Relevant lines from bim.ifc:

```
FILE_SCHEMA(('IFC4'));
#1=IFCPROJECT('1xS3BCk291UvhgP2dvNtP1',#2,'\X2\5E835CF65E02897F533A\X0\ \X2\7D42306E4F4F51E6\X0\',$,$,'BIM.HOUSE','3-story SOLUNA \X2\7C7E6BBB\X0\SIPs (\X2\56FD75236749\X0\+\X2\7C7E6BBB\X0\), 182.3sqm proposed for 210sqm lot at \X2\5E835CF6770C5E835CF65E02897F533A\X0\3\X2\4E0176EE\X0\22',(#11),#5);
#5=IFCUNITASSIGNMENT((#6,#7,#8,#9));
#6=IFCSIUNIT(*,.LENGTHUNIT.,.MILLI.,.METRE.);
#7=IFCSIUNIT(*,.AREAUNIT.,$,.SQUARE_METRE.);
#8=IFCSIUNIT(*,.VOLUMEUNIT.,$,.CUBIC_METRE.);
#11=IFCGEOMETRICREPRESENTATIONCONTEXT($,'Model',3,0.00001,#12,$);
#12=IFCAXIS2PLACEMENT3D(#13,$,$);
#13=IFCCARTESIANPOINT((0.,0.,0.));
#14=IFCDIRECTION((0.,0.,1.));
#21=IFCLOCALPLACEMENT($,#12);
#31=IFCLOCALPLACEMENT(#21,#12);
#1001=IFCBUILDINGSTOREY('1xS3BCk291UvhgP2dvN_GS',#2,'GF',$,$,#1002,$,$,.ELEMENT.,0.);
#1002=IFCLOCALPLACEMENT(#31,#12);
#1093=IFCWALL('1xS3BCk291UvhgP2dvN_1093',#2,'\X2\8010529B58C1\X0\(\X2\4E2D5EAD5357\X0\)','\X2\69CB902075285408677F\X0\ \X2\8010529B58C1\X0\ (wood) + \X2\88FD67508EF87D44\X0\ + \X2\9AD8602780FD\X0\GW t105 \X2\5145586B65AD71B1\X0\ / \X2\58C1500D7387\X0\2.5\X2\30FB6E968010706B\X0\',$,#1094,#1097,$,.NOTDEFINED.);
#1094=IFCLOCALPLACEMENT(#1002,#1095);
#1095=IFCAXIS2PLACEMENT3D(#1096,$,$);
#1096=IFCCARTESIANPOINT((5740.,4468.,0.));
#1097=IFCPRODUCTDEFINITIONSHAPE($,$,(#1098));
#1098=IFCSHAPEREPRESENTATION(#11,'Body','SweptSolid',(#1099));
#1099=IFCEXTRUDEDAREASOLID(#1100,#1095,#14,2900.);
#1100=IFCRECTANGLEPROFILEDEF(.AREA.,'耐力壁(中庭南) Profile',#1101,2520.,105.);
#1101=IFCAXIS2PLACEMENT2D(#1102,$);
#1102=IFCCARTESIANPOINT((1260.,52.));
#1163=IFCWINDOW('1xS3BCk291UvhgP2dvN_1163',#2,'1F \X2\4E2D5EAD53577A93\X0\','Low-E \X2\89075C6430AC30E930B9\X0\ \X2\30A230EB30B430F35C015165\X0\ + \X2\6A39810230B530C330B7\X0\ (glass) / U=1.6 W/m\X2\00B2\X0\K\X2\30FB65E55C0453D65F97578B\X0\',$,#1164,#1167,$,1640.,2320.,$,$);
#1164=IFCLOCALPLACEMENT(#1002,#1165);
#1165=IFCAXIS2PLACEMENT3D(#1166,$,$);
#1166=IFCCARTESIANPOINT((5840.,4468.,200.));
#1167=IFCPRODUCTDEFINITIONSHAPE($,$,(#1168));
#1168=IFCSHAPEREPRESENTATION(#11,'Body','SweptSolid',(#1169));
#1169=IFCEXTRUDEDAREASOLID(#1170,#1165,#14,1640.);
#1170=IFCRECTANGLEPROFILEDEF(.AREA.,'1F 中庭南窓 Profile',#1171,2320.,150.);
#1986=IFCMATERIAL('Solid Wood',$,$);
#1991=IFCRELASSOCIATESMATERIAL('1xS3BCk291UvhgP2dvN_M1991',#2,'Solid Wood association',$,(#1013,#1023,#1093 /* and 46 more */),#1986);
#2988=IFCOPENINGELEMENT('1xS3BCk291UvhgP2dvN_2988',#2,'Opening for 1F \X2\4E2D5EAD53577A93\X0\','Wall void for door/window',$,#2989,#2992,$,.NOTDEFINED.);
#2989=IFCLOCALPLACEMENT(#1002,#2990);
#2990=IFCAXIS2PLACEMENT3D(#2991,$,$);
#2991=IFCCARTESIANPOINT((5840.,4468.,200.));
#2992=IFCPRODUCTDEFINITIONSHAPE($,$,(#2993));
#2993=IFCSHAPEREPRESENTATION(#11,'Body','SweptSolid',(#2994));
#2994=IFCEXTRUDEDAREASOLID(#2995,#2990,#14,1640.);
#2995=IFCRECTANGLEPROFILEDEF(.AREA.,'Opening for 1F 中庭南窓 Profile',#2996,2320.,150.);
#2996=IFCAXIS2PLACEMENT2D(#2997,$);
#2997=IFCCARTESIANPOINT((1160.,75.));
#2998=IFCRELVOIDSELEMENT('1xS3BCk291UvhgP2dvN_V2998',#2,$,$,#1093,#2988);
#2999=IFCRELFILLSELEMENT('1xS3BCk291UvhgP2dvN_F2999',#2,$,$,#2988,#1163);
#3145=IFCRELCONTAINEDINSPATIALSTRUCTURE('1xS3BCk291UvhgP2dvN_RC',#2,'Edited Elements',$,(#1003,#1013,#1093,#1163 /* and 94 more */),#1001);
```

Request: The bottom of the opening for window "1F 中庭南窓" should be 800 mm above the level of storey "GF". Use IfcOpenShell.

```python
import numpy as np
import ifcopenshell
import ifcopenshell.api.geometry
import ifcopenshell.geom
import ifcopenshell.util.element
import ifcopenshell.util.placement
import ifcopenshell.util.shape
import ifcopenshell.util.unit

model = ifcopenshell.open("bim.ifc")
unit_scale = ifcopenshell.util.unit.calculate_unit_scale(model)

window = model.by_guid("1xS3BCk291UvhgP2dvN_1163")
opening = window.FillsVoids[0].RelatingOpeningElement
storey = ifcopenshell.util.element.get_container(window, ifc_class="IfcBuildingStorey")
level = ifcopenshell.util.placement.get_local_placement(storey.ObjectPlacement)[2, 3]

# The opening's origin need not be at the sill, so measure its lowest point.
shape = ifcopenshell.geom.create_shape(ifcopenshell.geom.settings(), opening)
bottom = ifcopenshell.util.shape.get_shape_bottom_elevation(shape, shape.geometry) / unit_scale
dz = level + 800.0 - bottom

shift = np.array([0.0, 0.0, dz])
# The window is not placed relative to its opening, so move both.
for product in (opening, window):
    matrix = ifcopenshell.util.placement.get_local_placement(product.ObjectPlacement)
    matrix[:3, 3] += shift
    ifcopenshell.api.geometry.edit_object_placement(model, product=product, matrix=matrix, is_si=False)

print(f"moved by {dz * unit_scale:+.3f} m")

model.write("bim-out.ifc")
```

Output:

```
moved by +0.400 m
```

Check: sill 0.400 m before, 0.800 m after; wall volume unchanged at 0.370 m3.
